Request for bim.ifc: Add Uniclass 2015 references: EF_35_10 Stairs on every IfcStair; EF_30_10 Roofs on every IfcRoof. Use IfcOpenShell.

First a look at what the model holds.

```python
import ifcopenshell

model = ifcopenshell.open("bim.ifc")
print(model.schema)
print("classifications:", [c.Name for c in model.by_type("IfcClassification")])
for ifc_class in ("IfcDoor", "IfcRoof", "IfcStair", "IfcWall", "IfcWindow"):
    print(ifc_class, len(model.by_type(ifc_class)))
```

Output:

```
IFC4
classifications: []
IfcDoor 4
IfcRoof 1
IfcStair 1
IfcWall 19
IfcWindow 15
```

```python
import ifcopenshell
import ifcopenshell.api.classification

model = ifcopenshell.open("bim.ifc")

system = ifcopenshell.api.classification.add_classification(model, classification="Uniclass 2015")

codes = {
    "IfcStair": ("EF_35_10", "Stairs"),
    "IfcRoof": ("EF_30_10", "Roofs"),
}
for ifc_class, (code, name) in codes.items():
    products = model.by_type(ifc_class)
    ifcopenshell.api.classification.add_reference(
        model, products=products, classification=system, identification=code, name=name
    )
    print(code, len(products))

model.write("bim-out.ifc")
```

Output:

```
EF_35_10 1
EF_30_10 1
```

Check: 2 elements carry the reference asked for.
